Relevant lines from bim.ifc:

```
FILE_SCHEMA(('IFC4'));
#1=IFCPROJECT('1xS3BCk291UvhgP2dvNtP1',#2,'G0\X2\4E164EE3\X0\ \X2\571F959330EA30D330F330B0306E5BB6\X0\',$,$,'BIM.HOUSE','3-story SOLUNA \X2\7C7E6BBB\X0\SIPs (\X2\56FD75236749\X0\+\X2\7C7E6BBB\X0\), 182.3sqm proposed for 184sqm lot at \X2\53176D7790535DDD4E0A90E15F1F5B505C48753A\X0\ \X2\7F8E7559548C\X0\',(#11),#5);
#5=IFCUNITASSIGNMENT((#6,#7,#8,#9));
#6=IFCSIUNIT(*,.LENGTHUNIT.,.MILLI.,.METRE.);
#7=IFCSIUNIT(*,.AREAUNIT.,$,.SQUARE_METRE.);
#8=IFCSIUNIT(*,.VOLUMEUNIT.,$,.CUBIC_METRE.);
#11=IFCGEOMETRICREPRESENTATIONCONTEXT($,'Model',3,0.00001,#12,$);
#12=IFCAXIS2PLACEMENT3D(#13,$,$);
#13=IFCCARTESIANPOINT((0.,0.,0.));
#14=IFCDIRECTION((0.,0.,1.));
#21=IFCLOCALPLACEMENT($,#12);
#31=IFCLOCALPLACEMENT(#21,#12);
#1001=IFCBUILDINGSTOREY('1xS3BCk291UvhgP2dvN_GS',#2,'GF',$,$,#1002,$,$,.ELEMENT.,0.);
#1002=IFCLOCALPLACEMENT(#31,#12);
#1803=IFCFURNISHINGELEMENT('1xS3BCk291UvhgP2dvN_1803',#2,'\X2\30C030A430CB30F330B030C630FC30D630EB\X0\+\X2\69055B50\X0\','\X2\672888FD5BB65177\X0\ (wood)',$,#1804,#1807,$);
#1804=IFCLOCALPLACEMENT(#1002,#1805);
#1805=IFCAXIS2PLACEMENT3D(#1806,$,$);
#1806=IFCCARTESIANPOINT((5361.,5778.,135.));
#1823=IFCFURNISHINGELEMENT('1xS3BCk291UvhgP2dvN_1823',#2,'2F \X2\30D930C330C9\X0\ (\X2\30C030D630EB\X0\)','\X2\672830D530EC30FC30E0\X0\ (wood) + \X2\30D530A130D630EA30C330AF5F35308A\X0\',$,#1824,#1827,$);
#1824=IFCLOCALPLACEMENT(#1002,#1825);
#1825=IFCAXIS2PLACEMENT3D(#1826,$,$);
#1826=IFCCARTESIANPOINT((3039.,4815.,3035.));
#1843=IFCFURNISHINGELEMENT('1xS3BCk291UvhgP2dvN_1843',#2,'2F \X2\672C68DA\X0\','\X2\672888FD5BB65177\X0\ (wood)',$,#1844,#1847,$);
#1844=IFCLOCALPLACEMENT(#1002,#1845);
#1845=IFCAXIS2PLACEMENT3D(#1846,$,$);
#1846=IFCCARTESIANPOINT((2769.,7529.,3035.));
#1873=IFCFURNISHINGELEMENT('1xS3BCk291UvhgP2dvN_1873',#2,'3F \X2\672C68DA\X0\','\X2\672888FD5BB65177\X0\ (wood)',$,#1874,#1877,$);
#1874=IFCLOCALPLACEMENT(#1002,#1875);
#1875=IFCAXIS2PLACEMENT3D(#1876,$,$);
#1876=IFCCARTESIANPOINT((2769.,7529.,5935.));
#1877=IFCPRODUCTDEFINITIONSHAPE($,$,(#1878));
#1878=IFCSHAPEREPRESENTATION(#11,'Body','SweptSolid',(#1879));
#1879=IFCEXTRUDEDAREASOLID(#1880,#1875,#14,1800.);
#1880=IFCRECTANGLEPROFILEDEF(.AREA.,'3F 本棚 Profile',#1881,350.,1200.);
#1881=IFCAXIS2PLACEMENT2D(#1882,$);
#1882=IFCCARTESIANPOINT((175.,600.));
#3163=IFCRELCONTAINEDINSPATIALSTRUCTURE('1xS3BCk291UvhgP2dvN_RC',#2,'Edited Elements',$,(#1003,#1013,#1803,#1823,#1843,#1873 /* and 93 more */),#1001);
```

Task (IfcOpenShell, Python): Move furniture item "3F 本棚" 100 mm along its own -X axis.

```python
import ifcopenshell
import ifcopenshell.api.geometry
import ifcopenshell.util.placement
import ifcopenshell.util.unit

model = ifcopenshell.open("bim.ifc")
unit_scale = ifcopenshell.util.unit.calculate_unit_scale(model)

item = model.by_id(1873)
matrix = ifcopenshell.util.placement.get_local_placement(item.ObjectPlacement)
matrix[:3, 3] -= matrix[:3, 0] * 0.1 / unit_scale
ifcopenshell.api.geometry.edit_object_placement(model, product=item, matrix=matrix, is_si=False)

print(ifcopenshell.util.placement.get_local_placement(item.ObjectPlacement).round(3) + 0.0)

model.write("bim_updated.ifc")
```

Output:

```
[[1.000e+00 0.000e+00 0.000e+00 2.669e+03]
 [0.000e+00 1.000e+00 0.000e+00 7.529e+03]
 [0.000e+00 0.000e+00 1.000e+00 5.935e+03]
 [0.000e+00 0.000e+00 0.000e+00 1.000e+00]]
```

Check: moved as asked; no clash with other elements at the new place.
